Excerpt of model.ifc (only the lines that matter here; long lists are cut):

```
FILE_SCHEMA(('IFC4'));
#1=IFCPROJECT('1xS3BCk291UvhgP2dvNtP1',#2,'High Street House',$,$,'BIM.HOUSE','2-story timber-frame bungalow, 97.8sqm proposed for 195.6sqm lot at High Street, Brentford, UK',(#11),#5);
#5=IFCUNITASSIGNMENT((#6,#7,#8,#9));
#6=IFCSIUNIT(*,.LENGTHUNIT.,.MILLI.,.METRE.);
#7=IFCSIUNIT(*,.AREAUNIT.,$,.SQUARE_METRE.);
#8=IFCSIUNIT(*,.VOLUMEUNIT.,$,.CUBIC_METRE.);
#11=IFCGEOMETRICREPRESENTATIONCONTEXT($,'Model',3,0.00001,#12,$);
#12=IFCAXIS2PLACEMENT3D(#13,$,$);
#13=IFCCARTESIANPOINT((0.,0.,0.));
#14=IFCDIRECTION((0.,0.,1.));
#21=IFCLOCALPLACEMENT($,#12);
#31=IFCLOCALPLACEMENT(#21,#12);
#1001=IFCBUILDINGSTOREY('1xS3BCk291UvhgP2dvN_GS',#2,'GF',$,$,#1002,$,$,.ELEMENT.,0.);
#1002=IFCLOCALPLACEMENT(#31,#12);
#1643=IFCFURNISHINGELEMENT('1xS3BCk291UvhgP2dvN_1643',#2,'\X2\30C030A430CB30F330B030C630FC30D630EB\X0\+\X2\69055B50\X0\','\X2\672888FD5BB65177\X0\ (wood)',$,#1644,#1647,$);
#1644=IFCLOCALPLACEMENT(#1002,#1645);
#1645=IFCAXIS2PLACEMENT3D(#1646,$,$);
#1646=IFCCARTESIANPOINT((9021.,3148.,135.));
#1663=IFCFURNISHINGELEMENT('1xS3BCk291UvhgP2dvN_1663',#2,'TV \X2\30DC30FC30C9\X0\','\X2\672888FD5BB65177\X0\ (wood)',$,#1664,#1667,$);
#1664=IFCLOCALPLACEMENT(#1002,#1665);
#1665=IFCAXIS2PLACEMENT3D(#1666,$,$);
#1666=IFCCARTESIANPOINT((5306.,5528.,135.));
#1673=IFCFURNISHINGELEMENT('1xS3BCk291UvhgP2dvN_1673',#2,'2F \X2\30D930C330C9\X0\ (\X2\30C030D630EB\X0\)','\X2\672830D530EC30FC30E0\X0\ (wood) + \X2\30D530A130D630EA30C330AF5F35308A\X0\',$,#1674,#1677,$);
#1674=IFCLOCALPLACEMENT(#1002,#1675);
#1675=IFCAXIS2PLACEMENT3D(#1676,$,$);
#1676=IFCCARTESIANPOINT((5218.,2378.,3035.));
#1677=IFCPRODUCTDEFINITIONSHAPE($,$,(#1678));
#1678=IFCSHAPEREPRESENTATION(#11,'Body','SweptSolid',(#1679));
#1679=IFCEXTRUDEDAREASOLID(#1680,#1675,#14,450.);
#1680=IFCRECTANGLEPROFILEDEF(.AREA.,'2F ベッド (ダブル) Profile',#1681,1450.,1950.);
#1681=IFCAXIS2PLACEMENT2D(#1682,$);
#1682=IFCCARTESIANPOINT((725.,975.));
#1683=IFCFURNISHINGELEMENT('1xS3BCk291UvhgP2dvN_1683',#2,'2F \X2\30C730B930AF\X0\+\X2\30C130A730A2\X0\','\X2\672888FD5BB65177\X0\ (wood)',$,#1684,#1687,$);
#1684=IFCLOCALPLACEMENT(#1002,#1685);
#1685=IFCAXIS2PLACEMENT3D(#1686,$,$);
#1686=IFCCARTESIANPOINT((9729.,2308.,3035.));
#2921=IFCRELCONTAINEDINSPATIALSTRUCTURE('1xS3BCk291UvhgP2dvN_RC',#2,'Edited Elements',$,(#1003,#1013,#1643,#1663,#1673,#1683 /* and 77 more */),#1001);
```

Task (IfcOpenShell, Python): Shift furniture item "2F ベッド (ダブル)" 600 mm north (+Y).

```python
import ifcopenshell
import ifcopenshell.api.geometry
import ifcopenshell.util.placement

model = ifcopenshell.open("model.ifc")

item = model.by_guid("1xS3BCk291UvhgP2dvN_1673")
matrix = ifcopenshell.util.placement.get_local_placement(item.ObjectPlacement)
matrix[1, 3] += 600.0
ifcopenshell.api.geometry.edit_object_placement(model, product=item, matrix=matrix, is_si=False)

print(ifcopenshell.util.placement.get_local_placement(item.ObjectPlacement).round(3) + 0.0)

model.write("model_updated.ifc")
```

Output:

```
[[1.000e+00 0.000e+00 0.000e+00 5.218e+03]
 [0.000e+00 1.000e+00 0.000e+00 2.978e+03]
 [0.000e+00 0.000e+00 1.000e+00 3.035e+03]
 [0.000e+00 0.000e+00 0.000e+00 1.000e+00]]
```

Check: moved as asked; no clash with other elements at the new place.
